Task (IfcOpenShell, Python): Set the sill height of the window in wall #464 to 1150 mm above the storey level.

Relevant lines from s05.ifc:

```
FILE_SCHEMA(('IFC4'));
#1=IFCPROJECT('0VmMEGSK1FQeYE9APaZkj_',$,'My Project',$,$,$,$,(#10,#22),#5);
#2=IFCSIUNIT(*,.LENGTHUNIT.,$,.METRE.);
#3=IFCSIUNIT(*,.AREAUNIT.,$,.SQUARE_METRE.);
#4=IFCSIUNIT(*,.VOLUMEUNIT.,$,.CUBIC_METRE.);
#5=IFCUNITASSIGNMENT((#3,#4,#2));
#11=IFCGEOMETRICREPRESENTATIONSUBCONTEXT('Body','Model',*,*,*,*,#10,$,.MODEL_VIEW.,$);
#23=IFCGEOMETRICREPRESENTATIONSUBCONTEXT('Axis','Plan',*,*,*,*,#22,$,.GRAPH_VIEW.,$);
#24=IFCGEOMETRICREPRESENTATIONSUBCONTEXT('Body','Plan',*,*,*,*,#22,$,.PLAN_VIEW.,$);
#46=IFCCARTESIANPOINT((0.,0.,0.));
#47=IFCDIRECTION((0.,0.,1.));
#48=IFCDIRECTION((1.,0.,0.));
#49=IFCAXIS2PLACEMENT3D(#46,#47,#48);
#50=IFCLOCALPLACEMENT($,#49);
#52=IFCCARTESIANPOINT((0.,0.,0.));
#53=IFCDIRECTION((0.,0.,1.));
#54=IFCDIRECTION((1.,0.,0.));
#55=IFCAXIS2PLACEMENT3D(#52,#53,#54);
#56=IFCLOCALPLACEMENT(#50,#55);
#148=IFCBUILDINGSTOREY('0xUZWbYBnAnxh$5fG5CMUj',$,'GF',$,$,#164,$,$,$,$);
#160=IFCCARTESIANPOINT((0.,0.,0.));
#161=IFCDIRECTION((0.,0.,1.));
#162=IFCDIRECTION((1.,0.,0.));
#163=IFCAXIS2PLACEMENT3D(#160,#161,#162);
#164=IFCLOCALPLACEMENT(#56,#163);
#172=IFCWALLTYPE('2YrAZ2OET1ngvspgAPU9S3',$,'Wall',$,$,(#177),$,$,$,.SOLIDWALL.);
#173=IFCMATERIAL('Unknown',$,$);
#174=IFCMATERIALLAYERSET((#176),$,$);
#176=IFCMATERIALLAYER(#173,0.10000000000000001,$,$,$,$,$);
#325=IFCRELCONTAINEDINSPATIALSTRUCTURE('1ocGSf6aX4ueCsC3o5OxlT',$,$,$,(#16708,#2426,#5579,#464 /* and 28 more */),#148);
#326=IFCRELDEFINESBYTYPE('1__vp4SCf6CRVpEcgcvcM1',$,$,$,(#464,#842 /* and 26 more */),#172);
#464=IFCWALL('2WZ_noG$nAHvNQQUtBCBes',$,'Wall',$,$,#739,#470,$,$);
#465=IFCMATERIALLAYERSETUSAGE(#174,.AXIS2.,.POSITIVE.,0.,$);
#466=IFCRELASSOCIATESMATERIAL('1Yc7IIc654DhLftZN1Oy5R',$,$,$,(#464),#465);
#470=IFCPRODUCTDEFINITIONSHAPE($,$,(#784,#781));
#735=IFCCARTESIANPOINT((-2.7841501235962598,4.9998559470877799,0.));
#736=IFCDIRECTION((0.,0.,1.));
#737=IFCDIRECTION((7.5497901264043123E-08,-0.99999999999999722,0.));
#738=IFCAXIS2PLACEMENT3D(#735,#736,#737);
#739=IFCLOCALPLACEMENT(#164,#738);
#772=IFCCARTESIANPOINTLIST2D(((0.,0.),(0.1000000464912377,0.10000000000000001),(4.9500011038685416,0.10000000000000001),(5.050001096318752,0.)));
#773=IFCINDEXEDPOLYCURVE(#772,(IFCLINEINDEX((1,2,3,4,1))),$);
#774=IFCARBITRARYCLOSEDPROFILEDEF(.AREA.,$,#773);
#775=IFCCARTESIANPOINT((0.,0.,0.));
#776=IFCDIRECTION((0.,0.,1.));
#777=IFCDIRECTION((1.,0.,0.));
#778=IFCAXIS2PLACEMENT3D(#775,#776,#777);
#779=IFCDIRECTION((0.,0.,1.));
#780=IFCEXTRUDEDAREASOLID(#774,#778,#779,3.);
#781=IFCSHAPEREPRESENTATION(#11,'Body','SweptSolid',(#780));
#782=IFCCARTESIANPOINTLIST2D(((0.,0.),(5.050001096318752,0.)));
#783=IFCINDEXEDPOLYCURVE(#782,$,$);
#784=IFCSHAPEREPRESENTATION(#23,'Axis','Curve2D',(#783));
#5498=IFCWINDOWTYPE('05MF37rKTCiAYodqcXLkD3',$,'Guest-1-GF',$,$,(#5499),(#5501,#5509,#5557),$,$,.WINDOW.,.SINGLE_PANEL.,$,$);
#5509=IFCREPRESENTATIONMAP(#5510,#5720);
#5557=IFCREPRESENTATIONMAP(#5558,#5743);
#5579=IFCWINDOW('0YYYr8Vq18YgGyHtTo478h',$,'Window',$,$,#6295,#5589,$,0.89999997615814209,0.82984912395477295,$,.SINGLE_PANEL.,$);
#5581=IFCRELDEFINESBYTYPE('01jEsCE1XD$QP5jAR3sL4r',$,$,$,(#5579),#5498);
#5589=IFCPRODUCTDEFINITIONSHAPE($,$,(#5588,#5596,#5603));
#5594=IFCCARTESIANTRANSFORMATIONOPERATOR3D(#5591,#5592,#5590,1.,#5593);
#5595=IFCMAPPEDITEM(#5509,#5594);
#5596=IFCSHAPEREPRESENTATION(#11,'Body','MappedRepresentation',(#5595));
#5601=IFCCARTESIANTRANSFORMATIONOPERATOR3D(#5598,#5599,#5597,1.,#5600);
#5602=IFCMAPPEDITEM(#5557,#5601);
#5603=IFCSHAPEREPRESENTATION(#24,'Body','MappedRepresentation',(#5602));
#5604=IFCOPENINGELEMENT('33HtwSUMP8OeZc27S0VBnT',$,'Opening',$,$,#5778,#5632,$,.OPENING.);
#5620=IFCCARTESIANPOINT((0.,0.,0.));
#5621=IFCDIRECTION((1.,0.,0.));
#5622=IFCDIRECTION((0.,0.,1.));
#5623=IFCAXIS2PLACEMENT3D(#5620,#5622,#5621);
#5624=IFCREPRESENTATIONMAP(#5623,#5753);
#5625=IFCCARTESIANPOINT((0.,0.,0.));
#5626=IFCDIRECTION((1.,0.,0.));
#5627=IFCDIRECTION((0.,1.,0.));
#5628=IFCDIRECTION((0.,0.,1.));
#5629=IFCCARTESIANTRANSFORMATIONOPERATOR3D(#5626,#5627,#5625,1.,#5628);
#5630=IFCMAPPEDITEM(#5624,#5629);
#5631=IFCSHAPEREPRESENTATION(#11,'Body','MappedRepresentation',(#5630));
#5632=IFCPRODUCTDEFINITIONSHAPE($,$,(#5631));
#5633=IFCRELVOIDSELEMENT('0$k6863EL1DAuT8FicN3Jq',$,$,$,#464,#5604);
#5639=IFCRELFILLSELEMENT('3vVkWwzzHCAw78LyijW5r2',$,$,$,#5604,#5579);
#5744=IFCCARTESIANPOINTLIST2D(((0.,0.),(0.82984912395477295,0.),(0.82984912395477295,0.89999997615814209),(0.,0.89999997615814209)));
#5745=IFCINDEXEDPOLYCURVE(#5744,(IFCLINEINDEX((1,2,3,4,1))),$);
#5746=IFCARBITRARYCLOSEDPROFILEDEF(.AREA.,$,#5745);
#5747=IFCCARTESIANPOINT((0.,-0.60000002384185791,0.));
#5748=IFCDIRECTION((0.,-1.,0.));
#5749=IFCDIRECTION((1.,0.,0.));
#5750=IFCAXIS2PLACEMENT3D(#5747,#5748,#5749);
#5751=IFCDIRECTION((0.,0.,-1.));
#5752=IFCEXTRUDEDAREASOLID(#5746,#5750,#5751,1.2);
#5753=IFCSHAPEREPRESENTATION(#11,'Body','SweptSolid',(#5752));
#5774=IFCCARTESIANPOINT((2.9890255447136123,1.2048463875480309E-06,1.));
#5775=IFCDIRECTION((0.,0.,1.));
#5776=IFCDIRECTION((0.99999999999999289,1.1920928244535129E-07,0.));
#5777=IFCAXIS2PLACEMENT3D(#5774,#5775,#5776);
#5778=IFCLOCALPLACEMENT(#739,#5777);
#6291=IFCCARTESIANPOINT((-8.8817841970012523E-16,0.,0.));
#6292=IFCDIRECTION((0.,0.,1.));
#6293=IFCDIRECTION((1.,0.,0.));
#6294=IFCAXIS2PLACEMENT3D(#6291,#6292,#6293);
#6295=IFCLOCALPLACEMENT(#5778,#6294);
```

```python
import numpy as np
import ifcopenshell
import ifcopenshell.api.geometry
import ifcopenshell.geom
import ifcopenshell.util.element
import ifcopenshell.util.placement
import ifcopenshell.util.shape
import ifcopenshell.util.unit

model = ifcopenshell.open("s05.ifc")
unit_scale = ifcopenshell.util.unit.calculate_unit_scale(model)

window = model.by_guid("0YYYr8Vq18YgGyHtTo478h")
opening = window.FillsVoids[0].RelatingOpeningElement
storey = ifcopenshell.util.element.get_container(window, ifc_class="IfcBuildingStorey")
level = ifcopenshell.util.placement.get_local_placement(storey.ObjectPlacement)[2, 3]

# The opening's origin need not be at the sill, so measure its lowest point.
shape = ifcopenshell.geom.create_shape(ifcopenshell.geom.settings(), opening)
bottom = ifcopenshell.util.shape.get_shape_bottom_elevation(shape, shape.geometry) / unit_scale
dz = level + 1.15 - bottom

shift = np.array([0.0, 0.0, dz])
# The window is placed relative to its opening, so it follows when the opening moves.
matrix = ifcopenshell.util.placement.get_local_placement(opening.ObjectPlacement)
matrix[:3, 3] += shift
ifcopenshell.api.geometry.edit_object_placement(
    model, product=opening, matrix=matrix, is_si=False, should_transform_children=True
)

print(f"moved by {dz * unit_scale:+.3f} m")

model.write("s05_updated.ifc")
```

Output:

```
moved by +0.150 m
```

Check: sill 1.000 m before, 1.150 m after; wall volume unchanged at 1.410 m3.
